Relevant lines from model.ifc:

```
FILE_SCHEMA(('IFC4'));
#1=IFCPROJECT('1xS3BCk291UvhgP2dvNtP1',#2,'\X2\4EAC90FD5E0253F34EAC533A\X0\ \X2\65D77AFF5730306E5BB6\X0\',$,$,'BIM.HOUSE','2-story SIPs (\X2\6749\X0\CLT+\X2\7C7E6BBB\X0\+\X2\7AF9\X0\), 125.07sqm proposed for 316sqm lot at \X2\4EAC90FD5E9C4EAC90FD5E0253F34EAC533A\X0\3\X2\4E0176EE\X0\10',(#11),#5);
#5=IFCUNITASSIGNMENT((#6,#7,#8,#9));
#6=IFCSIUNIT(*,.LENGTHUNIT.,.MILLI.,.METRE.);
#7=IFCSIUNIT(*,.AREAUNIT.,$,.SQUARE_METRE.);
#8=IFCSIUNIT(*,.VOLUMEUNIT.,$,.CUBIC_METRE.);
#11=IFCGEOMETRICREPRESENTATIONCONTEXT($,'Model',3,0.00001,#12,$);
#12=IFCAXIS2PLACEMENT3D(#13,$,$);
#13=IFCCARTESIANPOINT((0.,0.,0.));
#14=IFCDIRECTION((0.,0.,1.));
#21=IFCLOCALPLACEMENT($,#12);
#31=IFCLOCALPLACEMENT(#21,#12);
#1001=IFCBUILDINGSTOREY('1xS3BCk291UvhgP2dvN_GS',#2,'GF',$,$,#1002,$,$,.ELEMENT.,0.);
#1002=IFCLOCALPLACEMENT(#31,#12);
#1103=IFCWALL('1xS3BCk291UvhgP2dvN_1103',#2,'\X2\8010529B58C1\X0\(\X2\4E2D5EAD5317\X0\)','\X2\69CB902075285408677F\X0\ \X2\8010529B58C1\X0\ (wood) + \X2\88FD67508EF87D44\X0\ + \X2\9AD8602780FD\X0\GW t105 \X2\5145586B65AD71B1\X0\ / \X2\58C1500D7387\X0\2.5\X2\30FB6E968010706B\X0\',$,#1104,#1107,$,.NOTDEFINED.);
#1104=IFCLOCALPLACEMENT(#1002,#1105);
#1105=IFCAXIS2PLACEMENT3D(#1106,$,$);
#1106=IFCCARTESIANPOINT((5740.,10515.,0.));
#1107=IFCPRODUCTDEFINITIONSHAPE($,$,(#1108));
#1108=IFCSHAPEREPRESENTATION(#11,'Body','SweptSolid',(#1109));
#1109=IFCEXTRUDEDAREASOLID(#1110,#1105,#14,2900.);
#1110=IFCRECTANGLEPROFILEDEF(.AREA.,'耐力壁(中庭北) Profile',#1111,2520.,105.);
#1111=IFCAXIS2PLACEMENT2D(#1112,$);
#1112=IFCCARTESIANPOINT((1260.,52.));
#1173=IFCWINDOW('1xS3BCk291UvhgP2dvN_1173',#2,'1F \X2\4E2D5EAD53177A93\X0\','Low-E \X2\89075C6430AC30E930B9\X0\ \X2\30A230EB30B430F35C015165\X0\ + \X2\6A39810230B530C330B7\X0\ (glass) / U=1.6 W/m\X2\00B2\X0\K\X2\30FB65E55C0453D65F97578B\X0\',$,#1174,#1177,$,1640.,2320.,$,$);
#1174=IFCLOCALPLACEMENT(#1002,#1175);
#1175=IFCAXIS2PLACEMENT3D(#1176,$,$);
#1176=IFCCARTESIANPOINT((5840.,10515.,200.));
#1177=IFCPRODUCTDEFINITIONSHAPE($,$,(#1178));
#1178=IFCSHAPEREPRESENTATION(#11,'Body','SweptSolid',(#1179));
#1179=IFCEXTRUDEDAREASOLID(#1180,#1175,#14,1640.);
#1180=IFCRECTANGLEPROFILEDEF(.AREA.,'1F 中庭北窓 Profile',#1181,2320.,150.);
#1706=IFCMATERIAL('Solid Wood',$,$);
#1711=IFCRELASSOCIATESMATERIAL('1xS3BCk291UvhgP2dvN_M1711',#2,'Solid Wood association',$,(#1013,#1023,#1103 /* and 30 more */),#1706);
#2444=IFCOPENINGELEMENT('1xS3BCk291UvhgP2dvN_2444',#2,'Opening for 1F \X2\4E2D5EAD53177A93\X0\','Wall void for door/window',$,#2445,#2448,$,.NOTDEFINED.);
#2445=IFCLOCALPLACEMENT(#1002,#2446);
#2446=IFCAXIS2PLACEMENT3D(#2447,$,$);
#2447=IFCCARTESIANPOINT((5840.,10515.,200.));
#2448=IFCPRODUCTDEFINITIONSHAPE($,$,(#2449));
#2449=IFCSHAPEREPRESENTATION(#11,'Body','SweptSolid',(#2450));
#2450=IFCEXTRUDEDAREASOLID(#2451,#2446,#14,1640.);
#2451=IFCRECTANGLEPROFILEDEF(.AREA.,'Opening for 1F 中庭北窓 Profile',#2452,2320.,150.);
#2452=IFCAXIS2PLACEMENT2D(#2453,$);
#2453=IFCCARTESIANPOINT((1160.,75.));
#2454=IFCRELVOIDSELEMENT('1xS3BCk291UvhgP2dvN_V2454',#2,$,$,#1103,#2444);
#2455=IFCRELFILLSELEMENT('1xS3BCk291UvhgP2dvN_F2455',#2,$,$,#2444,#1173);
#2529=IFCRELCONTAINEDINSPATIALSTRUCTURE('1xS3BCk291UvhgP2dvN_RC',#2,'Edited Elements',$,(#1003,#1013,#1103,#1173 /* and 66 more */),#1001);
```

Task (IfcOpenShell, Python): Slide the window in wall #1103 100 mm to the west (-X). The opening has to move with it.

```python
import ifcopenshell
import ifcopenshell.api.geometry
import ifcopenshell.util.placement

model = ifcopenshell.open("model.ifc")

window = model.by_guid("1xS3BCk291UvhgP2dvN_1173")
opening = window.FillsVoids[0].RelatingOpeningElement
wall = opening.VoidsElements[0].RelatingBuildingElement

wall_matrix = ifcopenshell.util.placement.get_local_placement(wall.ObjectPlacement)
shift = wall_matrix[:3, 0] * -100.0
before = ifcopenshell.util.placement.get_local_placement(window.ObjectPlacement)[:3, 3].copy()

# The window is not placed relative to its opening, so move both.
for product in (opening, window):
    matrix = ifcopenshell.util.placement.get_local_placement(product.ObjectPlacement)
    matrix[:3, 3] += shift
    ifcopenshell.api.geometry.edit_object_placement(model, product=product, matrix=matrix, is_si=False)

after = ifcopenshell.util.placement.get_local_placement(window.ObjectPlacement)[:3, 3]
print("window moved by", (after - before).round(3) + 0.0)

model.write("model-out.ifc")
```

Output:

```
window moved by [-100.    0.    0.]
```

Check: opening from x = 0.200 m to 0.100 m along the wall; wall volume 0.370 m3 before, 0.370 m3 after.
